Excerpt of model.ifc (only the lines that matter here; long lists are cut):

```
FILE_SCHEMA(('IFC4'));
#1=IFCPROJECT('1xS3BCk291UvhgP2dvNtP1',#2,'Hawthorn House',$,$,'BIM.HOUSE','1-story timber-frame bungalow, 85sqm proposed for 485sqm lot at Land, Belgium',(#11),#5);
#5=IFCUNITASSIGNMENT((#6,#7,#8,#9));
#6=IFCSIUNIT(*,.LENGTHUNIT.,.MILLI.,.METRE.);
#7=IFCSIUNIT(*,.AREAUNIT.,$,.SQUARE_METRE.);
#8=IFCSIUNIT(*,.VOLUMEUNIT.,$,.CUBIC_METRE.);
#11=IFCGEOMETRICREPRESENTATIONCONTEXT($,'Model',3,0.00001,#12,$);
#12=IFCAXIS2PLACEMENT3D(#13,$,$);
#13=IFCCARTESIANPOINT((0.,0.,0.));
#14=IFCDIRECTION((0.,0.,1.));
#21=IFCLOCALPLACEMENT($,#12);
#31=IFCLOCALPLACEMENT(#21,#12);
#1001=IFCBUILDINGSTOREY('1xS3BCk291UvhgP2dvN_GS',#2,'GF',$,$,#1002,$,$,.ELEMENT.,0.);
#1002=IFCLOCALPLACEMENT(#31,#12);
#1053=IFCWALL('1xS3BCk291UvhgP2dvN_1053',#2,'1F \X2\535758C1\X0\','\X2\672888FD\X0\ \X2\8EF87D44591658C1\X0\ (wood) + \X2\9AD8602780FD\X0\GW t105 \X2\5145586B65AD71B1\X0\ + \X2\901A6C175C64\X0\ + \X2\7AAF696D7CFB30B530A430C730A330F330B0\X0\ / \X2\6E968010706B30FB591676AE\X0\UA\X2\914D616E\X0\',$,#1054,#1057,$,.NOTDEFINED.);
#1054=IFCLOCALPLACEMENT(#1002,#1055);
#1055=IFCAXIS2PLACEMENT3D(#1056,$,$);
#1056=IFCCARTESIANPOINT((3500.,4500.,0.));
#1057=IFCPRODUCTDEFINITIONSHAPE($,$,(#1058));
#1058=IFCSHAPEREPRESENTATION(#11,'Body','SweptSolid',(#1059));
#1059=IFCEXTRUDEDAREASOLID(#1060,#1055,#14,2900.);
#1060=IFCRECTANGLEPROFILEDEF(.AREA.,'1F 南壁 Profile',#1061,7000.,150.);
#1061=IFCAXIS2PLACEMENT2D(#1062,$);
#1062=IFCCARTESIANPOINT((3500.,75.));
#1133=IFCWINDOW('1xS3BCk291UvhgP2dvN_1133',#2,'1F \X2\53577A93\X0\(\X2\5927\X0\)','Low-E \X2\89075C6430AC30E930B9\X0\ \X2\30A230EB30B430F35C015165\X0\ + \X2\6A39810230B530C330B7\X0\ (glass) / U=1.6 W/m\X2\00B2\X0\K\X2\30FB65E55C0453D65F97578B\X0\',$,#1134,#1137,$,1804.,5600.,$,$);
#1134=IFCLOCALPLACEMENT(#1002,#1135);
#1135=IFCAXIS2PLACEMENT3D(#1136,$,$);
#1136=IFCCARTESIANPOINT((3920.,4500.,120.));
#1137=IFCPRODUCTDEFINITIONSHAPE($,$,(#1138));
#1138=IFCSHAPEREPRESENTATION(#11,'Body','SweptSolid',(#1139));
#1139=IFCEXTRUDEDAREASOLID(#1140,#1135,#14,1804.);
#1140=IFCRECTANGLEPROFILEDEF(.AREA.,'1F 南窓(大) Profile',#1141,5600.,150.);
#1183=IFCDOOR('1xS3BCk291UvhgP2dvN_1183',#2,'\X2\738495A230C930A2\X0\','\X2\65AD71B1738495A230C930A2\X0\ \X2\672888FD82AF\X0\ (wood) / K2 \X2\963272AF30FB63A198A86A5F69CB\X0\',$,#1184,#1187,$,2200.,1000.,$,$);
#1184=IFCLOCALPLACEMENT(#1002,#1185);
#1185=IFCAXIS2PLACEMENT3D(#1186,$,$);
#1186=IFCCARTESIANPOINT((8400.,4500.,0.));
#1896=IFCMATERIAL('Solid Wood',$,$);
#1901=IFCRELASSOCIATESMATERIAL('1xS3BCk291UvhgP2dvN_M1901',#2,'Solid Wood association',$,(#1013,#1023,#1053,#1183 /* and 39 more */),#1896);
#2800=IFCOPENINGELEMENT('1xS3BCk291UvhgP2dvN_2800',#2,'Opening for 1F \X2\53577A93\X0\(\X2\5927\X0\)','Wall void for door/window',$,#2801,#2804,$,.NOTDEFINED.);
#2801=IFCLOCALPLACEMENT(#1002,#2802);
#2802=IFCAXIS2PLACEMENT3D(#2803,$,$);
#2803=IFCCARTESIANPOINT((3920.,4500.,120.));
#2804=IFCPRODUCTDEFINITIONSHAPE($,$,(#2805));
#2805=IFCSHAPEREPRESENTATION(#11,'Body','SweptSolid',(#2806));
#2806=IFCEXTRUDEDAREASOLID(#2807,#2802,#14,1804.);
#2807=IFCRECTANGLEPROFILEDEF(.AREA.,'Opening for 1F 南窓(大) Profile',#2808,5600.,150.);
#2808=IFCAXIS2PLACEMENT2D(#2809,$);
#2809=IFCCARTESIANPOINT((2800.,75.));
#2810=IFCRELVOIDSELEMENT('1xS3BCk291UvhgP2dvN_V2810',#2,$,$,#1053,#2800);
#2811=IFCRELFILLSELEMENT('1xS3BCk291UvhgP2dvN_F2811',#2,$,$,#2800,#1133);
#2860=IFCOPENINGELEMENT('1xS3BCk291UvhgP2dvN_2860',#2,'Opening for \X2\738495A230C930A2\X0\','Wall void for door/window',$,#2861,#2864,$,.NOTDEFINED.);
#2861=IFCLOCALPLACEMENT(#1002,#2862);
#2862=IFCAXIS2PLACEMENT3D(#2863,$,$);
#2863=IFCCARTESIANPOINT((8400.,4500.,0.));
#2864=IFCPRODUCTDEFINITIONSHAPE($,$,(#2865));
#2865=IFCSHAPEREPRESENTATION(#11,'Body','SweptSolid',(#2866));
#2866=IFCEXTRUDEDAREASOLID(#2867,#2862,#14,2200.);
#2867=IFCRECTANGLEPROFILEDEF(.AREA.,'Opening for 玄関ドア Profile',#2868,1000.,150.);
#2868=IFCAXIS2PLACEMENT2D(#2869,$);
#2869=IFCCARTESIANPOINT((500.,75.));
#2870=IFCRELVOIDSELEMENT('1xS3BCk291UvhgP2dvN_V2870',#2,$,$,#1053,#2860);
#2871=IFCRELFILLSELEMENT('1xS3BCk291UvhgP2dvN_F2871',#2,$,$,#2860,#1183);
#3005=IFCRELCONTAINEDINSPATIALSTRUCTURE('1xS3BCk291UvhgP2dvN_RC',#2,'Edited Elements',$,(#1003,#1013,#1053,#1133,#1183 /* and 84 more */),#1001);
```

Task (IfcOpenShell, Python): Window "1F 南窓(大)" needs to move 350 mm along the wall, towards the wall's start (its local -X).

```python
import ifcopenshell
import ifcopenshell.api.geometry
import ifcopenshell.util.placement
import ifcopenshell.util.unit

model = ifcopenshell.open("model.ifc")
unit_scale = ifcopenshell.util.unit.calculate_unit_scale(model)

window = model.by_id(1133)
opening = window.FillsVoids[0].RelatingOpeningElement
wall = opening.VoidsElements[0].RelatingBuildingElement

wall_matrix = ifcopenshell.util.placement.get_local_placement(wall.ObjectPlacement)
shift = wall_matrix[:3, 0] * -0.35 / unit_scale
before = ifcopenshell.util.placement.get_local_placement(window.ObjectPlacement)[:3, 3].copy()

# The window is not placed relative to its opening, so move both.
for product in (opening, window):
    matrix = ifcopenshell.util.placement.get_local_placement(product.ObjectPlacement)
    matrix[:3, 3] += shift
    ifcopenshell.api.geometry.edit_object_placement(model, product=product, matrix=matrix, is_si=False)

after = ifcopenshell.util.placement.get_local_placement(window.ObjectPlacement)[:3, 3]
print("window moved by", (after - before).round(3) + 0.0)

model.write("model_edited.ifc")
```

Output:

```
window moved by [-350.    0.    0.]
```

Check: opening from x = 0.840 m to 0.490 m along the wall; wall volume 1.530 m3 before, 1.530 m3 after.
